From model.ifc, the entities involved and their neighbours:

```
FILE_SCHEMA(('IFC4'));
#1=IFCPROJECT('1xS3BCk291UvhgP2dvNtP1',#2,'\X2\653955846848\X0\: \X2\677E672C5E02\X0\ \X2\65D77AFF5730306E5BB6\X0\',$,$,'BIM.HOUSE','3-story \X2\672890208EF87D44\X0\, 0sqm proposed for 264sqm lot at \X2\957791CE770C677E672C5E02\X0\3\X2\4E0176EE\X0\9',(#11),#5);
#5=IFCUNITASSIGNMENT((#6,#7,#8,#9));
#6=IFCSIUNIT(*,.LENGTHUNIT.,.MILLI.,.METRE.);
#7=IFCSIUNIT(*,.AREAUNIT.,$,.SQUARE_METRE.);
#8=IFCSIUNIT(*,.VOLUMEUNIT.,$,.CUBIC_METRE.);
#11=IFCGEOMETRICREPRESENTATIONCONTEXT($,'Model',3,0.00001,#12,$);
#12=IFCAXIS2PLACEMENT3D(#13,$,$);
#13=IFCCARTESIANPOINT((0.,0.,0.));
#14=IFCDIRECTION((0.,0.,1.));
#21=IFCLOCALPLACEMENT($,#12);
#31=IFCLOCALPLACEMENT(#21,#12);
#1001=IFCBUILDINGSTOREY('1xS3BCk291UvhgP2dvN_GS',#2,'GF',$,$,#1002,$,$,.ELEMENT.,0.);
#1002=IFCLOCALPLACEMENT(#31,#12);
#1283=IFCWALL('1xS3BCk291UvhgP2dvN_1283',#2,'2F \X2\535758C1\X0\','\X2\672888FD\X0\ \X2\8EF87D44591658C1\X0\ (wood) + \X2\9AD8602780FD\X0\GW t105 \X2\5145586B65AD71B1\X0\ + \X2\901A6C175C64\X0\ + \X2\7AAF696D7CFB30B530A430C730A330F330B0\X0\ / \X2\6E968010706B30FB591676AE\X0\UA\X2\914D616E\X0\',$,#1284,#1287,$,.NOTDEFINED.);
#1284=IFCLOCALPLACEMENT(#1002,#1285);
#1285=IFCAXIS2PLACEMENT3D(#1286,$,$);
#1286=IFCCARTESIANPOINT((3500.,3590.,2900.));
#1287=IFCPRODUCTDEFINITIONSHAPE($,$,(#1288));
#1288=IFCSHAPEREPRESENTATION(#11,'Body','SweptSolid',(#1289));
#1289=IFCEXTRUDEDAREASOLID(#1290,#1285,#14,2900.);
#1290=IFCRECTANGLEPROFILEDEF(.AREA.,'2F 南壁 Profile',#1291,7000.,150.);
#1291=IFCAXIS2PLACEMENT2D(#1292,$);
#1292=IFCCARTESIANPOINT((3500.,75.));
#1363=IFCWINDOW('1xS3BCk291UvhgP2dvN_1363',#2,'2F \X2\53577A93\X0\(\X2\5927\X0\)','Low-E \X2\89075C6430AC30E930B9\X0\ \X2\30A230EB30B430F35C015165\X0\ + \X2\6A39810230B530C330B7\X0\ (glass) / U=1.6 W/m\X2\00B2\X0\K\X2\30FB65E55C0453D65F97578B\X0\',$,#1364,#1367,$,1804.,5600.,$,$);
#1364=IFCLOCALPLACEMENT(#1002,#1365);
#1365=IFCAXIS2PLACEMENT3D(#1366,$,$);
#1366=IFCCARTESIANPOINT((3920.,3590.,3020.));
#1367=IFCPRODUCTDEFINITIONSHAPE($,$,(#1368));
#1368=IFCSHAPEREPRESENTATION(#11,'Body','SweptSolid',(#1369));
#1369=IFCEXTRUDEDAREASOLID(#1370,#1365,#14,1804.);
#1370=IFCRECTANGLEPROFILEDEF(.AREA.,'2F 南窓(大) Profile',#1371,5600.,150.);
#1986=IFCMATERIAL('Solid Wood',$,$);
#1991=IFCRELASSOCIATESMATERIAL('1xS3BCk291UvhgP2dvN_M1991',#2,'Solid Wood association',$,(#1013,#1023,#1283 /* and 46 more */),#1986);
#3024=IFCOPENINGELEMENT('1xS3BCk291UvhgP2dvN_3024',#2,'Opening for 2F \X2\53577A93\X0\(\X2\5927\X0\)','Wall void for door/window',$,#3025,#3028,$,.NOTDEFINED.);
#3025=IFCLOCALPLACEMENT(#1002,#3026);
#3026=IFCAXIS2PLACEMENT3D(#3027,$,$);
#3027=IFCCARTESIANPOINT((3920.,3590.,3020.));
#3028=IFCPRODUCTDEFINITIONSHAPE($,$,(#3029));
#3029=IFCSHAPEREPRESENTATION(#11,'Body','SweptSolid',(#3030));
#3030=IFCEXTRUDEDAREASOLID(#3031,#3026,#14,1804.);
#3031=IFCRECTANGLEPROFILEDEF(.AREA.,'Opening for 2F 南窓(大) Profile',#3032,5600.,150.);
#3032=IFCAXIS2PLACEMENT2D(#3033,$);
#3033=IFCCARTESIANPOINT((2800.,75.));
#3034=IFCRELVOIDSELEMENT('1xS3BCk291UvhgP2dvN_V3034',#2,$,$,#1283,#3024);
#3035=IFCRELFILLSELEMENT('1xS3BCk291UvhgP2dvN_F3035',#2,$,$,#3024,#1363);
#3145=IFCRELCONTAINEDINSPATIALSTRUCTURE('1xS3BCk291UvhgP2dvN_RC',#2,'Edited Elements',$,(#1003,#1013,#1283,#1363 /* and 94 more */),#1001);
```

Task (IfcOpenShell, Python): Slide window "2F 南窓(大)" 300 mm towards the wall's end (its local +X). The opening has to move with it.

```python
import ifcopenshell
import ifcopenshell.api.geometry
import ifcopenshell.util.placement
import ifcopenshell.util.unit

model = ifcopenshell.open("model.ifc")
unit_scale = ifcopenshell.util.unit.calculate_unit_scale(model)

window = model.by_id(1363)
opening = window.FillsVoids[0].RelatingOpeningElement
wall = opening.VoidsElements[0].RelatingBuildingElement

wall_matrix = ifcopenshell.util.placement.get_local_placement(wall.ObjectPlacement)
shift = wall_matrix[:3, 0] * 0.3 / unit_scale
before = ifcopenshell.util.placement.get_local_placement(window.ObjectPlacement)[:3, 3].copy()

# The window is not placed relative to its opening, so move both.
for product in (opening, window):
    matrix = ifcopenshell.util.placement.get_local_placement(product.ObjectPlacement)
    matrix[:3, 3] += shift
    ifcopenshell.api.geometry.edit_object_placement(model, product=product, matrix=matrix, is_si=False)

after = ifcopenshell.util.placement.get_local_placement(window.ObjectPlacement)[:3, 3]
print("window moved by", (after - before).round(3) + 0.0)

model.write("model_rev.ifc")
```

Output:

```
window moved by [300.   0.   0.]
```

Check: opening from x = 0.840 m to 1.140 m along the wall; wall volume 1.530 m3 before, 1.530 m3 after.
